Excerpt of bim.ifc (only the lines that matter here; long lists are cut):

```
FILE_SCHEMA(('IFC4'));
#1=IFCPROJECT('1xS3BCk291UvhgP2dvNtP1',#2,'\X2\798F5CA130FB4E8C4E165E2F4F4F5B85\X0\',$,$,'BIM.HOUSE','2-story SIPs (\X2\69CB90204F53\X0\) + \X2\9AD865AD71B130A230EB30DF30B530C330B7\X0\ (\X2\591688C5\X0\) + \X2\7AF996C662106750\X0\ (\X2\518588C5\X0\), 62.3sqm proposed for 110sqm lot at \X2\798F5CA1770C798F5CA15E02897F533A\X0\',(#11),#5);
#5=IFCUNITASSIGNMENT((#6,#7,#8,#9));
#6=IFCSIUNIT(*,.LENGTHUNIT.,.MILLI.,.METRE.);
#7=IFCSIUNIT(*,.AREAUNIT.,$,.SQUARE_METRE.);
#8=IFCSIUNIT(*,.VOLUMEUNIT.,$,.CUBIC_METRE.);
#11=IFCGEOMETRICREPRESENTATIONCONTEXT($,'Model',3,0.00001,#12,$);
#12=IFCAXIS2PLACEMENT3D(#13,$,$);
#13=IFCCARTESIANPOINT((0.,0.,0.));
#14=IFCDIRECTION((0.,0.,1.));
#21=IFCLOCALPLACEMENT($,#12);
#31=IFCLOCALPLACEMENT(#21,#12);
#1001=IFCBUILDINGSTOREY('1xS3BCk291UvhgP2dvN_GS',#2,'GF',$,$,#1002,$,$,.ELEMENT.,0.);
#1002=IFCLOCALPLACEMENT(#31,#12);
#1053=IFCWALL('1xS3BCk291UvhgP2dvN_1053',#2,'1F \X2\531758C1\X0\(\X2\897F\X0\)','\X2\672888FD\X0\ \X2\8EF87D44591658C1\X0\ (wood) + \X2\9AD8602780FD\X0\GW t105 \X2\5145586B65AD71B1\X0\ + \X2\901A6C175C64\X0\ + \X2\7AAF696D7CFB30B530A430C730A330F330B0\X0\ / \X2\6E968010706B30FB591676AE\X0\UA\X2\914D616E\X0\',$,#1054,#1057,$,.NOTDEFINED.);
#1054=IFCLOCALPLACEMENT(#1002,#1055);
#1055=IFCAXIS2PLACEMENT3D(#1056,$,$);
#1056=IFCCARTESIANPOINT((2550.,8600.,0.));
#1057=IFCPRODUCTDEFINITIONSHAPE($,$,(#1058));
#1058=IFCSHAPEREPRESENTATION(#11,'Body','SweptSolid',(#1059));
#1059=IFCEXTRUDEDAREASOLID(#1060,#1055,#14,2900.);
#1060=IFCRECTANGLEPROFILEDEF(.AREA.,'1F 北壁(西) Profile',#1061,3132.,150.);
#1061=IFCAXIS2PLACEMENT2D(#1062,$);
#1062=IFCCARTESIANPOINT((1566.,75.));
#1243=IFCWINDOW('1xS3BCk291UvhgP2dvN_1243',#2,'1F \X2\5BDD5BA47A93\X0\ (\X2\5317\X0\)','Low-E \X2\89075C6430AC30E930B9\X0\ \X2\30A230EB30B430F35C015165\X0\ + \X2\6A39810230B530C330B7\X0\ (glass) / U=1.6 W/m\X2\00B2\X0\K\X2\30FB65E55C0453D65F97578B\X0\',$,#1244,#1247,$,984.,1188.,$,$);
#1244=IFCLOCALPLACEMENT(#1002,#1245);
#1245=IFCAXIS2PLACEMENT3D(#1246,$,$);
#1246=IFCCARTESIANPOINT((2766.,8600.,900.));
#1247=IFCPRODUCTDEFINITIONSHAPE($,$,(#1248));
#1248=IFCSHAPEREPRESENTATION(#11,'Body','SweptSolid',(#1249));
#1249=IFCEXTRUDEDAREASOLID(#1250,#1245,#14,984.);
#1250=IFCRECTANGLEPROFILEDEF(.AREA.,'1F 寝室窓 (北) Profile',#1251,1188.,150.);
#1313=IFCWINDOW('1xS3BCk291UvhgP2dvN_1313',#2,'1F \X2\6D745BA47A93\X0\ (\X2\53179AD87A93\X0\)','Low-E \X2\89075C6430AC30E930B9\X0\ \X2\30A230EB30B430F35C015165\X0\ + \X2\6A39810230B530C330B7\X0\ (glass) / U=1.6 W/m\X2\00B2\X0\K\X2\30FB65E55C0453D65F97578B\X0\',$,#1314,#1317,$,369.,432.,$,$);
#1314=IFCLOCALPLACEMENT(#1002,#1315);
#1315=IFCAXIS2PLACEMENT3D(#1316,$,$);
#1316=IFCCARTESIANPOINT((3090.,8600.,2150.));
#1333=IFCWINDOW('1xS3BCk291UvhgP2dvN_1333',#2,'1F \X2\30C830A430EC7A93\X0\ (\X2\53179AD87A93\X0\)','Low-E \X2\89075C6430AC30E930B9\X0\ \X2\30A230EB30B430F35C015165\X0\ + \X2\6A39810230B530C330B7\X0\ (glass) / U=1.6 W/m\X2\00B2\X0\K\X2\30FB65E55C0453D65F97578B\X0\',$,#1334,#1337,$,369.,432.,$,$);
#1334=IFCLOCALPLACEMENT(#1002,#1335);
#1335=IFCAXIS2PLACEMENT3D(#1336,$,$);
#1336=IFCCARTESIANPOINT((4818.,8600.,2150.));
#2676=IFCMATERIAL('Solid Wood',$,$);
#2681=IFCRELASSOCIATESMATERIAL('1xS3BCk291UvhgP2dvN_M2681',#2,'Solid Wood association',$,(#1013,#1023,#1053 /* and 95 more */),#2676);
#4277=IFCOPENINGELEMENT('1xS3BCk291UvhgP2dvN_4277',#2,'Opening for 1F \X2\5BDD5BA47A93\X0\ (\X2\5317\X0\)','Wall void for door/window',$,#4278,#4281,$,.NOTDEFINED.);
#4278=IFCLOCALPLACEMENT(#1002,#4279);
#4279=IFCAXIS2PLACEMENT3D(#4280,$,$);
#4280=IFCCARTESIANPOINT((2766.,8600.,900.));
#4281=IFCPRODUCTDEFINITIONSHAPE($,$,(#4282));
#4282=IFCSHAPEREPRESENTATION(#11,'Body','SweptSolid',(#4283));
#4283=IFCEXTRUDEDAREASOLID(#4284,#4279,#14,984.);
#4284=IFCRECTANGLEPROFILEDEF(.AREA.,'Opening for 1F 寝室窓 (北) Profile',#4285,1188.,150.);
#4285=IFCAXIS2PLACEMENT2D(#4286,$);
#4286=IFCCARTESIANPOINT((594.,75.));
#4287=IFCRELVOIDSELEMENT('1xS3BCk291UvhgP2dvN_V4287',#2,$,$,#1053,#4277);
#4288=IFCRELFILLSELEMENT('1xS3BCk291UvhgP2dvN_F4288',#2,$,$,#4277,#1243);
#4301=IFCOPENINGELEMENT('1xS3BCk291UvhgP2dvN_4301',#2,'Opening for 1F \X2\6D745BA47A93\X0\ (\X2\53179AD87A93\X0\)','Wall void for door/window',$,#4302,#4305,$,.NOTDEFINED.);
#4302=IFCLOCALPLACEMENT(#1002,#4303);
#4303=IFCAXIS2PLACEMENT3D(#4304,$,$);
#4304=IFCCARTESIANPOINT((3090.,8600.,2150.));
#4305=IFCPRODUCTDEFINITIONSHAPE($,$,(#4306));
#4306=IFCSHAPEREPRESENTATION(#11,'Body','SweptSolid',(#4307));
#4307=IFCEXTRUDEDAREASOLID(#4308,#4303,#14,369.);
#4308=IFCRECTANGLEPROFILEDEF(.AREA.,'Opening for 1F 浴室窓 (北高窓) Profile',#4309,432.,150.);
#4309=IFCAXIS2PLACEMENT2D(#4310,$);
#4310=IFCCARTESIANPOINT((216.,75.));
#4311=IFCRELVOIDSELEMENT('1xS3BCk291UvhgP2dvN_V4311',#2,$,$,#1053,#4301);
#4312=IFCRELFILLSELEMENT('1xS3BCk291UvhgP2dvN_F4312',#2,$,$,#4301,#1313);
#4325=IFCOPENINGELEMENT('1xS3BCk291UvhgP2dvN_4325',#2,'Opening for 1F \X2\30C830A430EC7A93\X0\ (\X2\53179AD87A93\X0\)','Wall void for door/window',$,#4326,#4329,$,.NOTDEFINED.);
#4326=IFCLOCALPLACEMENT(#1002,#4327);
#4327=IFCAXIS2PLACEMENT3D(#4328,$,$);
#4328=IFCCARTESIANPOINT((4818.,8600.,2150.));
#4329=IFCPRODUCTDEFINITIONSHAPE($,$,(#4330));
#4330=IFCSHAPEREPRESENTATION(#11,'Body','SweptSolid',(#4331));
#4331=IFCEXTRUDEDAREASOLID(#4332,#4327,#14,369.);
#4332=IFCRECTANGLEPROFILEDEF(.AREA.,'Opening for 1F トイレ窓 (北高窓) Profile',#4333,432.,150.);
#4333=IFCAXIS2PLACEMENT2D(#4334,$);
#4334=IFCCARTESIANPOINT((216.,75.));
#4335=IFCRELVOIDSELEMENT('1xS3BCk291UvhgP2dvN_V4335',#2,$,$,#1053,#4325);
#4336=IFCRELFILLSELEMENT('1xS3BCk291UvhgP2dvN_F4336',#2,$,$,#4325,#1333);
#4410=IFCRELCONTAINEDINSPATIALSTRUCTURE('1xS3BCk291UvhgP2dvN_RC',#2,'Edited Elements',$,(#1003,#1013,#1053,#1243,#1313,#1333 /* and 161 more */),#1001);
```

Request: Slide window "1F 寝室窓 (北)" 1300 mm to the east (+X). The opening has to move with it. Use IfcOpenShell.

```python
import ifcopenshell
import ifcopenshell.api.geometry
import ifcopenshell.util.placement
import ifcopenshell.util.unit

model = ifcopenshell.open("bim.ifc")
unit_scale = ifcopenshell.util.unit.calculate_unit_scale(model)

window = model.by_guid("1xS3BCk291UvhgP2dvN_1243")
opening = window.FillsVoids[0].RelatingOpeningElement
wall = opening.VoidsElements[0].RelatingBuildingElement

wall_matrix = ifcopenshell.util.placement.get_local_placement(wall.ObjectPlacement)
shift = wall_matrix[:3, 0] * 1.3 / unit_scale
before = ifcopenshell.util.placement.get_local_placement(window.ObjectPlacement)[:3, 3].copy()

# The window is not placed relative to its opening, so move both.
for product in (opening, window):
    matrix = ifcopenshell.util.placement.get_local_placement(product.ObjectPlacement)
    matrix[:3, 3] += shift
    ifcopenshell.api.geometry.edit_object_placement(model, product=product, matrix=matrix, is_si=False)

after = ifcopenshell.util.placement.get_local_placement(window.ObjectPlacement)[:3, 3]
print("window moved by", (after - before).round(3) + 0.0)

model.write("bim_v2.ifc")
```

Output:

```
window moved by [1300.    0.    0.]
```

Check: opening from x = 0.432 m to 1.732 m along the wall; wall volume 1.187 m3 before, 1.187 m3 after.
